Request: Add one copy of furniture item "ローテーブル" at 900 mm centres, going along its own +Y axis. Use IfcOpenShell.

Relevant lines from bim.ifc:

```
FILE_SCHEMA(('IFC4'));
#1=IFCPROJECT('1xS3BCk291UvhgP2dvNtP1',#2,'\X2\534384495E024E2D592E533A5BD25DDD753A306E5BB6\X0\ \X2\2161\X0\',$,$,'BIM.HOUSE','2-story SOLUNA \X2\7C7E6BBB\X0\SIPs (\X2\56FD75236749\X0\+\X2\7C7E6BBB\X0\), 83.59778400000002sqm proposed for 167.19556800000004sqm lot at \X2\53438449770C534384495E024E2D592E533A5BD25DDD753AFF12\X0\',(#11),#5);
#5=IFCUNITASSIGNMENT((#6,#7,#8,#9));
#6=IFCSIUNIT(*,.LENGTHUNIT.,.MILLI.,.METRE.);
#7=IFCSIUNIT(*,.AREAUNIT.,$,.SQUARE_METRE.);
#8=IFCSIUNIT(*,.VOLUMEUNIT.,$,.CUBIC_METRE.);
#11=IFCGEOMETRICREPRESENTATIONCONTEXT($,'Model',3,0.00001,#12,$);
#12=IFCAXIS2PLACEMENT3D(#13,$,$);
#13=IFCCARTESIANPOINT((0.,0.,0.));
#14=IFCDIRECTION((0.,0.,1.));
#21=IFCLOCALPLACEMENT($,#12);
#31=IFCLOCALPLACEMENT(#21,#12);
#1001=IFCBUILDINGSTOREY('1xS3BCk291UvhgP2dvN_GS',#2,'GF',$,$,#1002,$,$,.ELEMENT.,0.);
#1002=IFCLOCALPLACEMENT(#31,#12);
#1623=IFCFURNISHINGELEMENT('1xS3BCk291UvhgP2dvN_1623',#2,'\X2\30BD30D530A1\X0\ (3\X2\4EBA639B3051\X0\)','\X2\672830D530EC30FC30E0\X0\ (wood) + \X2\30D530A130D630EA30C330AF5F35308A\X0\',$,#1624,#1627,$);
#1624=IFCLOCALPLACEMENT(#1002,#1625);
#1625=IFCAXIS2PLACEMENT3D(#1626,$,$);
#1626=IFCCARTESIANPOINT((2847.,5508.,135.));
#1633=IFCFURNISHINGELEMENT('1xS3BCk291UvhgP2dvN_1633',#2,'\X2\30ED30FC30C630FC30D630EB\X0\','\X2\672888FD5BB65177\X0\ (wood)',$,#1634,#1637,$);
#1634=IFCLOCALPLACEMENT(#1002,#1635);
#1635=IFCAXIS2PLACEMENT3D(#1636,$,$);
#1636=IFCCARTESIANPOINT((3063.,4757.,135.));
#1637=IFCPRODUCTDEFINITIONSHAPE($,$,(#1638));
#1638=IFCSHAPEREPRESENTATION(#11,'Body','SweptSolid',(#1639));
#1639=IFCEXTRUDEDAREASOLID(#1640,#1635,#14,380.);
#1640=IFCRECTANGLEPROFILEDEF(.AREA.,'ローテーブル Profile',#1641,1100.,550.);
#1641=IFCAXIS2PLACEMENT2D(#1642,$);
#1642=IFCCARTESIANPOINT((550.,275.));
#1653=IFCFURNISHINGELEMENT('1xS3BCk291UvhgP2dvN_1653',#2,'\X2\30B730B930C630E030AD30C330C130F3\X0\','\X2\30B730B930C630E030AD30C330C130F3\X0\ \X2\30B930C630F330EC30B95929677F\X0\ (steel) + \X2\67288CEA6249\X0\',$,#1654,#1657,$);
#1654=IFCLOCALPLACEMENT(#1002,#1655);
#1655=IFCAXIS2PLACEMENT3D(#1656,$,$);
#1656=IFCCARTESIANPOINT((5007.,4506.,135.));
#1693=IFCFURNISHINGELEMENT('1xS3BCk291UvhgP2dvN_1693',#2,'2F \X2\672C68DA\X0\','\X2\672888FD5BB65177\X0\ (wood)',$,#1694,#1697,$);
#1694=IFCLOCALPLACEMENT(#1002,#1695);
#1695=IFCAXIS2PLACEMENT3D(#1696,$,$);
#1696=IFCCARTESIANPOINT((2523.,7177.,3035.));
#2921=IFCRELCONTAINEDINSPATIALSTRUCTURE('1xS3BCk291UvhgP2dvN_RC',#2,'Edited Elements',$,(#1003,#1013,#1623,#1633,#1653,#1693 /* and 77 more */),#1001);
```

```python
import ifcopenshell
import ifcopenshell.api.geometry
import ifcopenshell.api.root
import ifcopenshell.util.element
import ifcopenshell.util.placement

model = ifcopenshell.open("bim.ifc")


def reuse_history(source, copy):
    """copy_class also copies each property set's owner history, people and application; keep the originals."""
    for rel in copy.IsDefinedBy:
        if rel.is_a("IfcRelDefinesByProperties") and (history := rel.RelatingPropertyDefinition.OwnerHistory):
            rel.RelatingPropertyDefinition.OwnerHistory = source.OwnerHistory
            ifcopenshell.util.element.remove_deep2(model, history)


source = model.by_id(1633)
base = ifcopenshell.util.placement.get_local_placement(source.ObjectPlacement)
step = base[:3, 1] * 900.0

for i in range(1, 2):
    copy = ifcopenshell.api.root.copy_class(model, product=source)
    copy.Representation = ifcopenshell.util.element.copy_deep(
        model, source.Representation, exclude=["IfcGeometricRepresentationContext", "IfcRepresentationMap"]
    )
    reuse_history(source, copy)
    matrix = base.copy()
    matrix[:3, 3] += i * step
    print("added at", matrix[:3, 3].round(3) + 0.0)
    ifcopenshell.api.geometry.edit_object_placement(model, product=copy, matrix=matrix, is_si=False)

model.write("bim_rev.ifc")
```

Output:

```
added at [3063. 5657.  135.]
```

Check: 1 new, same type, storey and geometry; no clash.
